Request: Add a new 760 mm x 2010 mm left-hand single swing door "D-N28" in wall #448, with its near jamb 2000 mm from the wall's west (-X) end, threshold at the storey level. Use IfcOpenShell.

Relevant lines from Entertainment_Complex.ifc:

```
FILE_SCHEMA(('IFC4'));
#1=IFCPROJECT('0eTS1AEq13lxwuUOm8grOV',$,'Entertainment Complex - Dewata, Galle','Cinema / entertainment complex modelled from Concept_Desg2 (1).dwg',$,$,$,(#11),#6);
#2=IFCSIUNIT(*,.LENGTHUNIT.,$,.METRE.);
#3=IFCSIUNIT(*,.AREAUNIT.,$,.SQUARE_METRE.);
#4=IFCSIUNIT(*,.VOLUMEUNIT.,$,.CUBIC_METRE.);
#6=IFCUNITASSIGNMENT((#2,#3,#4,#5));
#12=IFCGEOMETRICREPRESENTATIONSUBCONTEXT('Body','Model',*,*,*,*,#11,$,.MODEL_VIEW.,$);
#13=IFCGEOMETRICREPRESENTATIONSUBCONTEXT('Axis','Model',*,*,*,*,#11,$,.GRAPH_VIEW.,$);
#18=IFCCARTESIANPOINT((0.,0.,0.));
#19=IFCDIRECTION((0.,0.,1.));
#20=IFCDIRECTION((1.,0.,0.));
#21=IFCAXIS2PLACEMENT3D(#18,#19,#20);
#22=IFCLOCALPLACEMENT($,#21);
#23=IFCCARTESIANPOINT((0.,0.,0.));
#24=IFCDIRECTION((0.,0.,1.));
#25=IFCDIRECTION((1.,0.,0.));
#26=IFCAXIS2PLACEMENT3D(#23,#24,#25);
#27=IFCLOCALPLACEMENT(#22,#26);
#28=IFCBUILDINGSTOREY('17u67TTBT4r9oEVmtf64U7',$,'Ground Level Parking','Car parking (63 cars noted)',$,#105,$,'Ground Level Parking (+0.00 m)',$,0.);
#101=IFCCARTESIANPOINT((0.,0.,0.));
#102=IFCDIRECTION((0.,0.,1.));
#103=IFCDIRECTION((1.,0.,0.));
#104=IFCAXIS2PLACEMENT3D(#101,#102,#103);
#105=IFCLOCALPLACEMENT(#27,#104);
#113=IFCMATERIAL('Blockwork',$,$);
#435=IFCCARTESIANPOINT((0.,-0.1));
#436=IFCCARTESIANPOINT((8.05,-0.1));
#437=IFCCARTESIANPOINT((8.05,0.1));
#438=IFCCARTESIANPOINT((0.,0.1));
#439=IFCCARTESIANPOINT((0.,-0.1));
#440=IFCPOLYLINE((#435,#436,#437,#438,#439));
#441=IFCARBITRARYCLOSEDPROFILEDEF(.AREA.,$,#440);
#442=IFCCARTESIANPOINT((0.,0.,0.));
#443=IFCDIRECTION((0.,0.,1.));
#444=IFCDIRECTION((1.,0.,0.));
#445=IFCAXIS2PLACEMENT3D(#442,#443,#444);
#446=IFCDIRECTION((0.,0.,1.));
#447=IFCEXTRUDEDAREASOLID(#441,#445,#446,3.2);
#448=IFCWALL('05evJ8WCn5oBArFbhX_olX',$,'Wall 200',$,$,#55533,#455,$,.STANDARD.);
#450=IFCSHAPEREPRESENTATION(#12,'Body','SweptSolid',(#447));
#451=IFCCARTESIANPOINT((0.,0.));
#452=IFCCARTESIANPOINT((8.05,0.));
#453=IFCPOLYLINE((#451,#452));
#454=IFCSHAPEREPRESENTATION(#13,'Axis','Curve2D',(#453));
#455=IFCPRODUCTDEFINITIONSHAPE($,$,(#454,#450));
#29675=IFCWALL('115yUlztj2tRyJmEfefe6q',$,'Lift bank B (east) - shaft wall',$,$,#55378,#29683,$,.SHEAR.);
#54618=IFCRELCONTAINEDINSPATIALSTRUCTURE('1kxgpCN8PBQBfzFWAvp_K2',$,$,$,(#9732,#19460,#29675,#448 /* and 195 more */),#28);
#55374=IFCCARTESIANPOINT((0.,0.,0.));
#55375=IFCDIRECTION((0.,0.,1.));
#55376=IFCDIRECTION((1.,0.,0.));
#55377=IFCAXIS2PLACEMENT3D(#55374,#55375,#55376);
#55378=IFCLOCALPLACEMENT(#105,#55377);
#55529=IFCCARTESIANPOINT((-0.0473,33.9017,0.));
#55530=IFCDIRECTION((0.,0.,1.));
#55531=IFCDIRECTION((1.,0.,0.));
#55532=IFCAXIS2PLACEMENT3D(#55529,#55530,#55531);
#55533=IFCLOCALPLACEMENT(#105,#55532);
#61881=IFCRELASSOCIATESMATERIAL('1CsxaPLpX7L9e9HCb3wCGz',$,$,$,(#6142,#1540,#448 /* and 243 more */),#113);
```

```python
import numpy as np
import ifcopenshell
import ifcopenshell.api.feature
import ifcopenshell.api.geometry
import ifcopenshell.api.root
import ifcopenshell.api.spatial
import ifcopenshell.geom
import ifcopenshell.util.element
import ifcopenshell.util.placement
import ifcopenshell.util.representation
import ifcopenshell.util.shape
import ifcopenshell.util.unit

model = ifcopenshell.open("Entertainment_Complex.ifc")
unit_scale = ifcopenshell.util.unit.calculate_unit_scale(model)
settings = ifcopenshell.geom.settings()


def volume(element):
    """Net volume in cubic metres, openings subtracted."""
    shape = ifcopenshell.geom.create_shape(settings, element)
    return ifcopenshell.util.shape.get_volume(shape.geometry)


wall = model.by_guid("05evJ8WCn5oBArFbhX_olX")
storey = ifcopenshell.util.element.get_container(wall, ifc_class="IfcBuildingStorey")
context = ifcopenshell.util.representation.get_context(model, "Model", "Body", "MODEL_VIEW")
before = volume(wall)

width, height, from_end, sill = 0.76, 2.01, 2, 0.0  # metres

# The wall runs along its own X axis, and the end named is its -X end.
wall_shape = ifcopenshell.geom.create_shape(settings, wall)
x, y, z = ifcopenshell.util.shape.get_vertices(wall_shape.geometry).T
start = x.min() + from_end
face, thickness = float(y.min()), float(y.max() - y.min())
wall_matrix = ifcopenshell.util.placement.get_local_placement(wall.ObjectPlacement)
level = ifcopenshell.util.placement.get_local_placement(storey.ObjectPlacement)[2, 3]


def in_wall(x, y):
    """Placement at x, y metres in the wall's axes, at sill height."""
    matrix = wall_matrix.copy()
    matrix[:, 3] = wall_matrix @ np.array([x / unit_scale, y / unit_scale, 0.0, 1.0])
    matrix[2, 3] = level + sill / unit_scale
    return matrix


# Opening: a box that overshoots both wall faces by 50 mm.
opening = ifcopenshell.api.root.create_entity(model, ifc_class="IfcOpeningElement", predefined_type="OPENING")
box = ifcopenshell.api.geometry.add_wall_representation(
    model, context=context, length=width, height=height, thickness=thickness + 0.1
)
ifcopenshell.api.geometry.assign_representation(model, product=opening, representation=box)
ifcopenshell.api.geometry.edit_object_placement(model, product=opening, matrix=in_wall(start, face - 0.05), is_si=False)
ifcopenshell.api.feature.add_feature(model, feature=opening, element=wall)

door = ifcopenshell.api.root.create_entity(model, ifc_class="IfcDoor", name="D-N28", predefined_type="DOOR")
door.OverallWidth, door.OverallHeight = width / unit_scale, height / unit_scale
door.OperationType = "SINGLE_SWING_LEFT"
body = ifcopenshell.api.geometry.add_door_representation(
    model,
    context=context,
    overall_width=door.OverallWidth,
    overall_height=door.OverallHeight,
    operation_type="SINGLE_SWING_LEFT",
    lining_properties={"LiningDepth": thickness / unit_scale, "ThresholdDepth": thickness / unit_scale},
)
ifcopenshell.api.geometry.assign_representation(model, product=door, representation=body)
ifcopenshell.api.spatial.assign_container(model, products=[door], relating_structure=storey)
ifcopenshell.api.feature.add_filling(model, opening=opening, element=door)

# The lining spans the wall, so the door starts at the wall face.
ifcopenshell.api.geometry.edit_object_placement(model, product=door, matrix=in_wall(start, face), is_si=False)

after = volume(wall)

print(f"wall volume {before:.3f} -> {after:.3f} m3")

model.write("Entertainment_Complex_updated.ifc")
```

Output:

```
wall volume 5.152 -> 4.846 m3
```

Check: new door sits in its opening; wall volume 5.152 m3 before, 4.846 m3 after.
